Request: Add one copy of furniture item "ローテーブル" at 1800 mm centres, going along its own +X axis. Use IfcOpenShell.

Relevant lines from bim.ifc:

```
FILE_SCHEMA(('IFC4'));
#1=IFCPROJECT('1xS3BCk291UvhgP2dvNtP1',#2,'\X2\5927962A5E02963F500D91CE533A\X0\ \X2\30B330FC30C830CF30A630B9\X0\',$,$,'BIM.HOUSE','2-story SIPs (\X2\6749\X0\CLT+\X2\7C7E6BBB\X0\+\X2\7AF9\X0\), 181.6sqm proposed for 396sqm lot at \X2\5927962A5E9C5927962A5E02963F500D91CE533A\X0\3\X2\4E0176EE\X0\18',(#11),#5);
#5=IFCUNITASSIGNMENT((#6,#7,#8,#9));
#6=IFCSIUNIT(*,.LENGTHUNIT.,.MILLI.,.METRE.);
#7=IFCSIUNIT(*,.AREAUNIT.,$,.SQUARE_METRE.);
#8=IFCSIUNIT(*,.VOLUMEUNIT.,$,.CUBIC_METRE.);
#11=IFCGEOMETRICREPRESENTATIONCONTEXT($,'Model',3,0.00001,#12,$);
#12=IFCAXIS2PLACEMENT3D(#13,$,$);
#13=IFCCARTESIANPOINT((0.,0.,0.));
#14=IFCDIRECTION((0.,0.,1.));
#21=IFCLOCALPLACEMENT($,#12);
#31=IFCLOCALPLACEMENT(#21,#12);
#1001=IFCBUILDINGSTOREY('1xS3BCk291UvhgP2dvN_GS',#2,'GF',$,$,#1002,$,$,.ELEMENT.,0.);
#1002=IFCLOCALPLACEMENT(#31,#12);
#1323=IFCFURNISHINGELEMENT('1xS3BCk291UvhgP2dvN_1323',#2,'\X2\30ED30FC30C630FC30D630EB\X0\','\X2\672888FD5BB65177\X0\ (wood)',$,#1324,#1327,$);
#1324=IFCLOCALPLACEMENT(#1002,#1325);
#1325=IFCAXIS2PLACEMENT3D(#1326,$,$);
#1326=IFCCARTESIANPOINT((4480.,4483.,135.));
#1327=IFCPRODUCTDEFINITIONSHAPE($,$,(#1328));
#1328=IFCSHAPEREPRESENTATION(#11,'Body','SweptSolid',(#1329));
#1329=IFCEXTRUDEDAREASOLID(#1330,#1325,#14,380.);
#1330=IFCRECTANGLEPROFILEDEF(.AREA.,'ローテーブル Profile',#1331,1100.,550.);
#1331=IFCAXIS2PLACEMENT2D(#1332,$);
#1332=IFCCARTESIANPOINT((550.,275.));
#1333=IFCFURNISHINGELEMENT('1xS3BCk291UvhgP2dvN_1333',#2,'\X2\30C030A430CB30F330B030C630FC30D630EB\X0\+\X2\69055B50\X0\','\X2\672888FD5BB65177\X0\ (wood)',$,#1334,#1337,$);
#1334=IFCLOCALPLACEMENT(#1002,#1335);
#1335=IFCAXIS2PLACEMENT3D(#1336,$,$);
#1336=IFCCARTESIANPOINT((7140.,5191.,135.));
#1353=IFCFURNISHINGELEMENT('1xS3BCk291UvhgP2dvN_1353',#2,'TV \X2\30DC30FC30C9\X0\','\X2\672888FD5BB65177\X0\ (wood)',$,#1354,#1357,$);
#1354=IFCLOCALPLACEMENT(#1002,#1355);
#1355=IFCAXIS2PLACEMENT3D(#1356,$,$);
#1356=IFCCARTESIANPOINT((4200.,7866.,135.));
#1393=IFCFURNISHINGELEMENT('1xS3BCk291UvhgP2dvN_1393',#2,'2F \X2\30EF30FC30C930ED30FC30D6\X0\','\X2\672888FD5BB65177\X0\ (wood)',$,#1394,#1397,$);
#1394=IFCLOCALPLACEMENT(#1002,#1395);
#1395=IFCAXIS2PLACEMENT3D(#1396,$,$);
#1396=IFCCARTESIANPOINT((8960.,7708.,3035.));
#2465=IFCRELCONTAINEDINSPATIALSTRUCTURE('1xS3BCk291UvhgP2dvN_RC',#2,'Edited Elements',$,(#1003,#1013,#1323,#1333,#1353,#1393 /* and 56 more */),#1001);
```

```python
import ifcopenshell
import ifcopenshell.api.geometry
import ifcopenshell.api.root
import ifcopenshell.util.element
import ifcopenshell.util.placement

model = ifcopenshell.open("bim.ifc")


def reuse_history(source, copy):
    """copy_class also copies each property set's owner history, people and application; keep the originals."""
    for rel in copy.IsDefinedBy:
        if rel.is_a("IfcRelDefinesByProperties") and (history := rel.RelatingPropertyDefinition.OwnerHistory):
            rel.RelatingPropertyDefinition.OwnerHistory = source.OwnerHistory
            ifcopenshell.util.element.remove_deep2(model, history)


source = model.by_guid("1xS3BCk291UvhgP2dvN_1323")
base = ifcopenshell.util.placement.get_local_placement(source.ObjectPlacement)
step = base[:3, 0] * 1800.0

for i in range(1, 2):
    copy = ifcopenshell.api.root.copy_class(model, product=source)
    copy.Representation = ifcopenshell.util.element.copy_deep(
        model, source.Representation, exclude=["IfcGeometricRepresentationContext", "IfcRepresentationMap"]
    )
    reuse_history(source, copy)
    matrix = base.copy()
    matrix[:3, 3] += i * step
    print("added at", matrix[:3, 3].round(3) + 0.0)
    ifcopenshell.api.geometry.edit_object_placement(model, product=copy, matrix=matrix, is_si=False)

model.write("bim_v2.ifc")
```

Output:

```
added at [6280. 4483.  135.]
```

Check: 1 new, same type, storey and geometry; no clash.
